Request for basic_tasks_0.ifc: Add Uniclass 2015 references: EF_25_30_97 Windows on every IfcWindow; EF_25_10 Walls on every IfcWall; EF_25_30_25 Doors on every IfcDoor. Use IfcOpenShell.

First a look at what the model holds.

```python
import ifcopenshell

model = ifcopenshell.open("basic_tasks_0.ifc")
print(model.schema)
print("classifications:", [c.Name for c in model.by_type("IfcClassification")])
for ifc_class in ("IfcDoor", "IfcRoof", "IfcStair", "IfcWall", "IfcWindow"):
    print(ifc_class, len(model.by_type(ifc_class)))
```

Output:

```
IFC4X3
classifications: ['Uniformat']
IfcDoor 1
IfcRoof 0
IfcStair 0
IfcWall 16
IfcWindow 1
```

```python
import ifcopenshell
import ifcopenshell.api.classification

model = ifcopenshell.open("basic_tasks_0.ifc")

system = ifcopenshell.api.classification.add_classification(model, classification="Uniclass 2015")

codes = {
    "IfcWindow": ("EF_25_30_97", "Windows"),
    "IfcWall": ("EF_25_10", "Walls"),
    "IfcDoor": ("EF_25_30_25", "Doors"),
}
for ifc_class, (code, name) in codes.items():
    products = model.by_type(ifc_class)
    ifcopenshell.api.classification.add_reference(
        model, products=products, classification=system, identification=code, name=name
    )
    print(code, len(products))

model.write("basic_tasks_0_rev.ifc")
```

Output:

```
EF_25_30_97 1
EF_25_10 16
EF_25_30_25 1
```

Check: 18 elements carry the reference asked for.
